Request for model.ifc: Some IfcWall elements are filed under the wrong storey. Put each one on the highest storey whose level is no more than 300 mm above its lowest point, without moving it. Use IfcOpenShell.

First a look at what the model holds.

```python
import ifcopenshell
import ifcopenshell.util.element
import ifcopenshell.util.placement

model = ifcopenshell.open("model.ifc")
print(model.schema)
for storey in model.by_type("IfcBuildingStorey"):
    level = ifcopenshell.util.placement.get_storey_elevation(storey)
    count = sum(e.is_a("IfcWall") for e in ifcopenshell.util.element.get_contained(storey))
    print(storey.id(), storey.Name, round(level, 3), count, sep=" | ")
```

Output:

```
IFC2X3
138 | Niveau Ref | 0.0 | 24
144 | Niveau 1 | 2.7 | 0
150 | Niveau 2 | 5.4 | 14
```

```python
import ifcopenshell
import ifcopenshell.api.spatial
import ifcopenshell.geom
import ifcopenshell.util.element
import ifcopenshell.util.placement
import ifcopenshell.util.shape
import ifcopenshell.util.unit

model = ifcopenshell.open("model.ifc")
unit_scale = ifcopenshell.util.unit.calculate_unit_scale(model)
settings = ifcopenshell.geom.settings()

levels = sorted(
    ((ifcopenshell.util.placement.get_storey_elevation(s) * unit_scale, s) for s in model.by_type("IfcBuildingStorey")),
    key=lambda pair: pair[0],
)

for e in model.by_type("IfcWall"):
    current = e.ContainedInStructure[0].RelatingStructure if e.ContainedInStructure else None
    if current is None or not current.is_a("IfcBuildingStorey"):
        continue
    shape = ifcopenshell.geom.create_shape(settings, e)
    bottom = ifcopenshell.util.shape.get_shape_bottom_elevation(shape, shape.geometry)
    below = [s for level, s in levels if level <= bottom + 0.3]
    storey = below[-1] if below else levels[0][1]
    if storey != current:
        # assign_container keeps the world position.
        ifcopenshell.api.spatial.assign_container(model, products=[e], relating_structure=storey)
        print(e.id(), current.Name, "->", storey.Name)

model.write("model_rev.ifc")
```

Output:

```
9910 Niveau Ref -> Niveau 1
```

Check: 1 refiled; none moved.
